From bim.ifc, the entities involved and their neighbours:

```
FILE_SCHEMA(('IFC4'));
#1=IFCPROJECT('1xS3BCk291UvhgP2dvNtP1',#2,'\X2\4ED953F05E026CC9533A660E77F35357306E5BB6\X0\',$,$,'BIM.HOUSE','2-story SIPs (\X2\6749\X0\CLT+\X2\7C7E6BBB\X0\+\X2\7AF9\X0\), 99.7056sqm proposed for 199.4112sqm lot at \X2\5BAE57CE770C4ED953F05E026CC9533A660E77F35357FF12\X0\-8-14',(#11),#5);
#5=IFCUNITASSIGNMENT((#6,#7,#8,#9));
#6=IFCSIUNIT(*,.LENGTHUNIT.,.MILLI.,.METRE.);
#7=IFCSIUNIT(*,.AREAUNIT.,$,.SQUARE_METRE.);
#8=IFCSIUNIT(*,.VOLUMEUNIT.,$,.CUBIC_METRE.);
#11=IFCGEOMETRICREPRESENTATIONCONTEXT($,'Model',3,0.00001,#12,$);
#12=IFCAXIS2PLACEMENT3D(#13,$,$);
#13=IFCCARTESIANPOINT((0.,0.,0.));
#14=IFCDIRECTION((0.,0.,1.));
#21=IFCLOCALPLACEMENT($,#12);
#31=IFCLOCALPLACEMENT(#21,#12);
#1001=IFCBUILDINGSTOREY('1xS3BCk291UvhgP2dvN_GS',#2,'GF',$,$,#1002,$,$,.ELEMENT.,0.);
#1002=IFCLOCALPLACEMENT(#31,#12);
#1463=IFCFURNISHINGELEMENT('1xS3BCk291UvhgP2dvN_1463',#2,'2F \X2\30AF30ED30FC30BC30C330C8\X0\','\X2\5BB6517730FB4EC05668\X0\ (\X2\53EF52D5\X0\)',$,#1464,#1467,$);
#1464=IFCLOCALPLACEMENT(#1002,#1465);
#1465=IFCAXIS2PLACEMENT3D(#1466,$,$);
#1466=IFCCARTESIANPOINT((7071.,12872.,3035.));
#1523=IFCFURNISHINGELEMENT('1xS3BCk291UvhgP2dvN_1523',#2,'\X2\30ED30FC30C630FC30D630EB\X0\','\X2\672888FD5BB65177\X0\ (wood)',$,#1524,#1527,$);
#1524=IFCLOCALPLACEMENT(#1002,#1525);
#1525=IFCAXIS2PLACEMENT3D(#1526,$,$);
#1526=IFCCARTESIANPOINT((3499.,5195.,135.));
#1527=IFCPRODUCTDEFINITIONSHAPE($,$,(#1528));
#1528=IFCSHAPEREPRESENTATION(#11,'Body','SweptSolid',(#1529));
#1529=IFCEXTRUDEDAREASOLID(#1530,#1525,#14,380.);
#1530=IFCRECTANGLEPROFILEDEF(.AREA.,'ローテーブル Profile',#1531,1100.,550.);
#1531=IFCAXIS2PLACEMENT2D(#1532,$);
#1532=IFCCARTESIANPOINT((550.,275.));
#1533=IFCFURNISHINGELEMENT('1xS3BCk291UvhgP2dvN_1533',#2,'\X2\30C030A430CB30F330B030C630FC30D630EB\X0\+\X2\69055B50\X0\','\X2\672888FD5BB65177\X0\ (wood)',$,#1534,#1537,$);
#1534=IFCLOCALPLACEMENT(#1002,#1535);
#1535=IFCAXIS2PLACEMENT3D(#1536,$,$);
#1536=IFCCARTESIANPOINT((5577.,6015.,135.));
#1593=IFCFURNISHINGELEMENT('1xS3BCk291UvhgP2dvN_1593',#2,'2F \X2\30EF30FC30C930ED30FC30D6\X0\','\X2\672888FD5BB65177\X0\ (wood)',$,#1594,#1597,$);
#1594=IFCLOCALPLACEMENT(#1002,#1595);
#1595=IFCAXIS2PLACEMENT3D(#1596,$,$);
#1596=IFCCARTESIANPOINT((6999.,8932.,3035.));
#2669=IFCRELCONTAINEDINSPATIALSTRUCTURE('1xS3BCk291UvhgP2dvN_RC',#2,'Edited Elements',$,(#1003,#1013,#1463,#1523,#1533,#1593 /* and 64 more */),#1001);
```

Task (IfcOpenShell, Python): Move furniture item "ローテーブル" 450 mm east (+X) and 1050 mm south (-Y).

```python
import ifcopenshell
import ifcopenshell.api.geometry
import ifcopenshell.util.placement
import ifcopenshell.util.unit

model = ifcopenshell.open("bim.ifc")
unit_scale = ifcopenshell.util.unit.calculate_unit_scale(model)

item = model.by_guid("1xS3BCk291UvhgP2dvN_1523")
matrix = ifcopenshell.util.placement.get_local_placement(item.ObjectPlacement)
matrix[0, 3] += 0.45 / unit_scale
matrix[1, 3] -= 1.05 / unit_scale
ifcopenshell.api.geometry.edit_object_placement(model, product=item, matrix=matrix, is_si=False)

print(ifcopenshell.util.placement.get_local_placement(item.ObjectPlacement).round(3) + 0.0)

model.write("bim_edited.ifc")
```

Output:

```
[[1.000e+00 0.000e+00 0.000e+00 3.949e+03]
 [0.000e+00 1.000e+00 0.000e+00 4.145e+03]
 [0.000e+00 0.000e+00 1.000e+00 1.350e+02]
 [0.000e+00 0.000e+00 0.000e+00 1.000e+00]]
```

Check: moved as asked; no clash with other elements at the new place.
